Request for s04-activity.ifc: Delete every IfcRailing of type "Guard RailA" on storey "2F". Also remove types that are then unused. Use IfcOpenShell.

First a look at what the model holds.

```python
import ifcopenshell
import ifcopenshell.util.element

model = ifcopenshell.open("s04-activity.ifc")
print(model.schema)
storey = next(s for s in model.by_type("IfcBuildingStorey") if s.Name == "2F")
railings = [e for e in ifcopenshell.util.element.get_decomposition(storey) if e.is_a("IfcRailing")]
seen = {}
for e in railings:
    element_type = ifcopenshell.util.element.get_type(e)
    name = element_type.Name if element_type not in (None, e) else None
    seen[name] = seen.get(name, 0) + 1
for name, count in sorted(seen.items(), key=str):
    print(count, "x", name)
```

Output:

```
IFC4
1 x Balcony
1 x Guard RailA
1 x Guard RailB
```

```python
import ifcopenshell
import ifcopenshell.api.root
import ifcopenshell.util.element

model = ifcopenshell.open("s04-activity.ifc")

storey = next(s for s in model.by_type("IfcBuildingStorey") if s.Name == "2F")
railings = [e for e in ifcopenshell.util.element.get_decomposition(storey) if e.is_a("IfcRailing")]
targets = [e for e in railings if (t := ifcopenshell.util.element.get_type(e)) not in (None, e) and t.Name == "Guard RailA"]
types = {ifcopenshell.util.element.get_type(e) for e in targets} - {None, *targets}

for e in targets:
    ifcopenshell.api.root.remove_product(model, product=e)
print(len(targets), "removed")

unused = [t for t in types if not ifcopenshell.util.element.get_types(t)]
for t in unused:
    ifcopenshell.api.root.remove_product(model, product=t)
print(len(unused), "unused types removed")

model.write("s04-activity_updated.ifc")
```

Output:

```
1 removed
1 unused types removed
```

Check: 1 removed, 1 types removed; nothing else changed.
